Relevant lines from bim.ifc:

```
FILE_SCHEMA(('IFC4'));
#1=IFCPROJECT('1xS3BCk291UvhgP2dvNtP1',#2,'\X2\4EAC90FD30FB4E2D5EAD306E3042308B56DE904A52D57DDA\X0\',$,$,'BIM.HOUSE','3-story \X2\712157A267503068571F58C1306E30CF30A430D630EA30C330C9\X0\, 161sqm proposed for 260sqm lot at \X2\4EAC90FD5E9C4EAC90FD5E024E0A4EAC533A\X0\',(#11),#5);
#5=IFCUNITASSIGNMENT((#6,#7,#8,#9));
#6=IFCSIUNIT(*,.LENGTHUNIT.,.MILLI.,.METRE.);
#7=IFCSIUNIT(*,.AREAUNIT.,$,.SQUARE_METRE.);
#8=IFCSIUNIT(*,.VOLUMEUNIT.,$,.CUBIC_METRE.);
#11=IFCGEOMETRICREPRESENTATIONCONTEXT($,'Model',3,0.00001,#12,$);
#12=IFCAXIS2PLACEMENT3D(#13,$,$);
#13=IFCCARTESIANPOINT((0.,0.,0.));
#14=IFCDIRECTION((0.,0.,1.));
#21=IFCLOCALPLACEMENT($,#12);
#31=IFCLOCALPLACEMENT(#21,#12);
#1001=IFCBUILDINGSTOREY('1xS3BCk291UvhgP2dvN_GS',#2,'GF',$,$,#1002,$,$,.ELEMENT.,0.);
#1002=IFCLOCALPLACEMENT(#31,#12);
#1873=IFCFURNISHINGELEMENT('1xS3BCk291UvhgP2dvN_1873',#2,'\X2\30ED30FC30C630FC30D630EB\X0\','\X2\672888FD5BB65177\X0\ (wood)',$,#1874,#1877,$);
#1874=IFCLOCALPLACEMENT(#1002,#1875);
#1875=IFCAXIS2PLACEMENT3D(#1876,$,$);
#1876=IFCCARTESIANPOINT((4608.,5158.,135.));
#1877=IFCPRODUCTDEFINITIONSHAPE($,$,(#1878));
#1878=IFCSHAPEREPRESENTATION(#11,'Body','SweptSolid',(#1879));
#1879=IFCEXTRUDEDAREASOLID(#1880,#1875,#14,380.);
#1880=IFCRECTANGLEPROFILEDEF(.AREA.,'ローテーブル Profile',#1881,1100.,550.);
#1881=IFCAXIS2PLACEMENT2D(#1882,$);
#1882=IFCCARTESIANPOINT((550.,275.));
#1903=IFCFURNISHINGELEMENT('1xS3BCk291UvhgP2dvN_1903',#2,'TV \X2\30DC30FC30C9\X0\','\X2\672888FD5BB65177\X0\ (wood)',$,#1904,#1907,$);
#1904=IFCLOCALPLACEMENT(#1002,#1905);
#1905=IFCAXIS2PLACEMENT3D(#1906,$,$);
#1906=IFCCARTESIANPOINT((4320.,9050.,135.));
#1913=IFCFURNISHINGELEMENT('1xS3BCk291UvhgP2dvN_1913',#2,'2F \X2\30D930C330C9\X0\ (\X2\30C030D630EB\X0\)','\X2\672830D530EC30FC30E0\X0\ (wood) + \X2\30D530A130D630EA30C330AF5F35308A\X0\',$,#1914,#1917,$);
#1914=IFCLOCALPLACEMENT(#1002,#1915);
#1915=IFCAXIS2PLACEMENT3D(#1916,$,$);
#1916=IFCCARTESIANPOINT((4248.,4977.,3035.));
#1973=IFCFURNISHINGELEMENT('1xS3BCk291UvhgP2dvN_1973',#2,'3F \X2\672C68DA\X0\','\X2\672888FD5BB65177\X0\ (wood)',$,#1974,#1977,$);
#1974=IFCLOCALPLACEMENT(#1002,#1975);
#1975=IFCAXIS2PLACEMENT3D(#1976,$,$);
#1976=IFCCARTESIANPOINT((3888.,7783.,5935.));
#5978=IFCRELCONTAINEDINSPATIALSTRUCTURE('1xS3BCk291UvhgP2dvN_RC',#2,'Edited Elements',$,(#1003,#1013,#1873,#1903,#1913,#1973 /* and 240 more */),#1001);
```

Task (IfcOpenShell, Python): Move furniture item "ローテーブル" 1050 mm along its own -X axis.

```python
import ifcopenshell
import ifcopenshell.api.geometry
import ifcopenshell.util.placement
import ifcopenshell.util.unit

model = ifcopenshell.open("bim.ifc")
unit_scale = ifcopenshell.util.unit.calculate_unit_scale(model)

item = model.by_guid("1xS3BCk291UvhgP2dvN_1873")
matrix = ifcopenshell.util.placement.get_local_placement(item.ObjectPlacement)
matrix[:3, 3] -= matrix[:3, 0] * 1.05 / unit_scale
ifcopenshell.api.geometry.edit_object_placement(model, product=item, matrix=matrix, is_si=False)

print(ifcopenshell.util.placement.get_local_placement(item.ObjectPlacement).round(3) + 0.0)

model.write("bim_v2.ifc")
```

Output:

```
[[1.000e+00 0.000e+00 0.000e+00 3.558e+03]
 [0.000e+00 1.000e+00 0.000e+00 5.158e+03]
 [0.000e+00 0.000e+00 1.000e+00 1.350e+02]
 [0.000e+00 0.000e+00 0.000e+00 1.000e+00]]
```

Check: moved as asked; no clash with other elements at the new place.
